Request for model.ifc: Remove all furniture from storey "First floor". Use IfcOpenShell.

First a look at what the model holds.

```python
import ifcopenshell
import ifcopenshell.util.element

model = ifcopenshell.open("model.ifc")
print(model.schema)
storey = next(s for s in model.by_type("IfcBuildingStorey") if s.Name == "First floor")
furniture = [e for e in ifcopenshell.util.element.get_decomposition(storey) if e.is_a("IfcFurnishingElement")]
seen = {}
for e in furniture:
    element_type = ifcopenshell.util.element.get_type(e)
    name = element_type.Name if element_type not in (None, e) else None
    seen[name] = seen.get(name, 0) + 1
for name, count in sorted(seen.items(), key=str):
    print(count, "x", name)
```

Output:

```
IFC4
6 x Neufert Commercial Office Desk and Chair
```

```python
import ifcopenshell
import ifcopenshell.api.root
import ifcopenshell.util.element

model = ifcopenshell.open("model.ifc")

storey = next(s for s in model.by_type("IfcBuildingStorey") if s.Name == "First floor")
furniture = [e for e in ifcopenshell.util.element.get_decomposition(storey) if e.is_a("IfcFurnishingElement")]

for e in furniture:
    ifcopenshell.api.root.remove_product(model, product=e)
print(len(furniture), "removed")

model.write("model_edited.ifc")
```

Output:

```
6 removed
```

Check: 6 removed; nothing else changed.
